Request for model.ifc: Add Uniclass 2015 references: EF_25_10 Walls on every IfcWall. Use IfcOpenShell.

First a look at what the model holds.

```python
import ifcopenshell

model = ifcopenshell.open("model.ifc")
print(model.schema)
print("classifications:", [c.Name for c in model.by_type("IfcClassification")])
for ifc_class in ("IfcDoor", "IfcRoof", "IfcStair", "IfcWall", "IfcWindow"):
    print(ifc_class, len(model.by_type(ifc_class)))
```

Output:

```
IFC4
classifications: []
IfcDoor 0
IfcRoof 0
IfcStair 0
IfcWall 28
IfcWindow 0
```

```python
import ifcopenshell
import ifcopenshell.api.classification

model = ifcopenshell.open("model.ifc")

system = ifcopenshell.api.classification.add_classification(model, classification="Uniclass 2015")

codes = {
    "IfcWall": ("EF_25_10", "Walls"),
}
for ifc_class, (code, name) in codes.items():
    products = model.by_type(ifc_class)
    ifcopenshell.api.classification.add_reference(
        model, products=products, classification=system, identification=code, name=name
    )
    print(code, len(products))

model.write("model_rev.ifc")
```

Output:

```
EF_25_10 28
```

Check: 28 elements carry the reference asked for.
